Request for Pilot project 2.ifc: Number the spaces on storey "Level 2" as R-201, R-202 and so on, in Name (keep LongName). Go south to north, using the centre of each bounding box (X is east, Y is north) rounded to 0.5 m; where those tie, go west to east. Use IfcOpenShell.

First a look at what the model holds.

```python
import ifcopenshell
import ifcopenshell.util.element
import ifcopenshell.util.placement

model = ifcopenshell.open("Pilot project 2.ifc")
print(model.schema)
storey = next(s for s in model.by_type("IfcBuildingStorey") if s.Name == "Level 2")
spaces = [e for e in ifcopenshell.util.element.get_decomposition(storey) if e.is_a("IfcSpace")]
for e in sorted(spaces, key=lambda e: e.id()):
    origin = ifcopenshell.util.placement.get_local_placement(e.ObjectPlacement)[:3, 3]
    print(e.id(), e.Name, e.LongName, origin.round(2) + 0.0, sep=" | ")
```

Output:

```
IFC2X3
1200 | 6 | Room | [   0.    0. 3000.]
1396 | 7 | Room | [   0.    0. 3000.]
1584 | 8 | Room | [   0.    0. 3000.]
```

```python
import ifcopenshell
import ifcopenshell.geom
import ifcopenshell.util.element
import ifcopenshell.util.shape

model = ifcopenshell.open("Pilot project 2.ifc")
settings = ifcopenshell.geom.settings()
settings.set("use-world-coords", True)


def centre(element):
    shape = ifcopenshell.geom.create_shape(settings, element)
    return ifcopenshell.util.shape.get_bbox_centroid(shape.geometry)


storey = next(s for s in model.by_type("IfcBuildingStorey") if s.Name == "Level 2")
spaces = [e for e in ifcopenshell.util.element.get_decomposition(storey) if e.is_a("IfcSpace")]

# Insertion points can sit at a corner or the storey origin, so sort by the geometry (in metres).
centres = {e: centre(e) for e in spaces}
spaces.sort(key=lambda e: (round(centres[e][1] / 0.5), centres[e][0]))

for i, e in enumerate(spaces, start=1):
    number = f"R-2{i:02d}"
    e.Name = number
    print(e.id(), number)

model.write("Pilot project 2_v2.ifc")
```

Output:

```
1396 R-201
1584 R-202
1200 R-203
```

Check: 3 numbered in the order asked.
